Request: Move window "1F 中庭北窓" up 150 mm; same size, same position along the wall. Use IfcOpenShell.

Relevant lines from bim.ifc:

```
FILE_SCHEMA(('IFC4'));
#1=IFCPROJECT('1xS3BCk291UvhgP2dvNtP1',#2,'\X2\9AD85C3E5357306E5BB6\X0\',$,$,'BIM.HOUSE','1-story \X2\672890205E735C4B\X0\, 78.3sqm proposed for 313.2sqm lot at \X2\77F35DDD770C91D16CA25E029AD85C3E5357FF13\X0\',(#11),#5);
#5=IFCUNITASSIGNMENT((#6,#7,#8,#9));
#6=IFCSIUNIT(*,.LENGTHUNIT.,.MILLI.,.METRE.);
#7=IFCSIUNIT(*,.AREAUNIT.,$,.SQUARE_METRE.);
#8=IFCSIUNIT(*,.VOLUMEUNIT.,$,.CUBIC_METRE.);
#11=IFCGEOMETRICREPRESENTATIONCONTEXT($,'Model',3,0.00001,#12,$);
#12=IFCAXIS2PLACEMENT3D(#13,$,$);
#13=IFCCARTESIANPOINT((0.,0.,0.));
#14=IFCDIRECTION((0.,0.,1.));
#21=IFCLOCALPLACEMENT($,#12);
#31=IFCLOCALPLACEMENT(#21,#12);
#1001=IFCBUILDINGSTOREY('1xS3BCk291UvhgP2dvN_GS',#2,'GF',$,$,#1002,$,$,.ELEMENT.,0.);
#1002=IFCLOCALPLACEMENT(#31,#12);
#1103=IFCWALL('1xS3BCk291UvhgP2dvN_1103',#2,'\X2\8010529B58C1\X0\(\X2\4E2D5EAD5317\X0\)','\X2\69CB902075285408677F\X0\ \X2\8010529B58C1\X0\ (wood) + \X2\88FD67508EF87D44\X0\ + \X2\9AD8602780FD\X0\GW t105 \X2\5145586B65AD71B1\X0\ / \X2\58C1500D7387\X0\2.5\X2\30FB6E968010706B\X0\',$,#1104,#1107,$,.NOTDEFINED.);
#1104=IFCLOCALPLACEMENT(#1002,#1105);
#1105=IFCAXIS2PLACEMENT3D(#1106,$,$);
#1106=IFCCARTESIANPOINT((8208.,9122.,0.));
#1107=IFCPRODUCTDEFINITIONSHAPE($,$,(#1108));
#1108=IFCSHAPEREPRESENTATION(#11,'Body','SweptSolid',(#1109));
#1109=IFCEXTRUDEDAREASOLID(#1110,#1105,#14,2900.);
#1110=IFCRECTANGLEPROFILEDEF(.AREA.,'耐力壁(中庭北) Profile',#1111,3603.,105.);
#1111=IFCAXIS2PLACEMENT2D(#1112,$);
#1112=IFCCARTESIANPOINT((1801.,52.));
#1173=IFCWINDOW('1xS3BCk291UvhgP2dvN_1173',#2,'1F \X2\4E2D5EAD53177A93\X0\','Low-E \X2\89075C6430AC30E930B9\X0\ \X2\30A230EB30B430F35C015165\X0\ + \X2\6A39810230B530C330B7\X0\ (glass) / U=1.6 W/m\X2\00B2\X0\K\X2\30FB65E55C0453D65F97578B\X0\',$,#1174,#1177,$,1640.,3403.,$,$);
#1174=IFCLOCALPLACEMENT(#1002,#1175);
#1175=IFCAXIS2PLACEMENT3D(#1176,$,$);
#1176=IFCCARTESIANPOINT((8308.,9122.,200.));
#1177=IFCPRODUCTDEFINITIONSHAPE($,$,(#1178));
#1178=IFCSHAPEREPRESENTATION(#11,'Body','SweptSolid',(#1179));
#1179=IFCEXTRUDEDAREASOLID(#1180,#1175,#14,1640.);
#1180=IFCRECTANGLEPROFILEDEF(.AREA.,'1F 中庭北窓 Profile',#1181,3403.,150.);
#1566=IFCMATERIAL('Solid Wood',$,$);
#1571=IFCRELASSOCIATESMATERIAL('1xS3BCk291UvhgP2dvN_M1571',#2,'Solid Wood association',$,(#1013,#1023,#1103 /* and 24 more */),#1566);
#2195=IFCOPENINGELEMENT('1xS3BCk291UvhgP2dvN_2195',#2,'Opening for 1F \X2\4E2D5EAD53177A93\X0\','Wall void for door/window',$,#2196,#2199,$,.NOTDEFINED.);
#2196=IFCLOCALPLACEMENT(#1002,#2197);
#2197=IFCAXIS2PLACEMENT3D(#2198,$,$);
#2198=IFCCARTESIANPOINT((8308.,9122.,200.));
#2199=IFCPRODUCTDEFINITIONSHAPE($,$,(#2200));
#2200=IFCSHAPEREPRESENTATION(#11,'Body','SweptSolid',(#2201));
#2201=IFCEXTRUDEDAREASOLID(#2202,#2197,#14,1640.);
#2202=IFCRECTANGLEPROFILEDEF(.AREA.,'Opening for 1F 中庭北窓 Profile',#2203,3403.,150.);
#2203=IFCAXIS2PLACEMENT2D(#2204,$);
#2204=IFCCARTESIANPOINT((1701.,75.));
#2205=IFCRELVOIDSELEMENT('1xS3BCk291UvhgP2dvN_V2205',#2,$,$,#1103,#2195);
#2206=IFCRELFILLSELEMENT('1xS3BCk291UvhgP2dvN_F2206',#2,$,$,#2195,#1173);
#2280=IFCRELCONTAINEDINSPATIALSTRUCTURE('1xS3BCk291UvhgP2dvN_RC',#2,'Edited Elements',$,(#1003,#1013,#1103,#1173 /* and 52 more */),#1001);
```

```python
import numpy as np
import ifcopenshell
import ifcopenshell.api.geometry
import ifcopenshell.util.placement
import ifcopenshell.util.unit

model = ifcopenshell.open("bim.ifc")
unit_scale = ifcopenshell.util.unit.calculate_unit_scale(model)

window = model.by_guid("1xS3BCk291UvhgP2dvN_1173")
opening = window.FillsVoids[0].RelatingOpeningElement
dz = 0.15 / unit_scale

shift = np.array([0.0, 0.0, dz])
# The window is not placed relative to its opening, so move both.
for product in (opening, window):
    matrix = ifcopenshell.util.placement.get_local_placement(product.ObjectPlacement)
    matrix[:3, 3] += shift
    ifcopenshell.api.geometry.edit_object_placement(model, product=product, matrix=matrix, is_si=False)

print(f"moved by {dz * unit_scale:+.3f} m")

model.write("bim_updated.ifc")
```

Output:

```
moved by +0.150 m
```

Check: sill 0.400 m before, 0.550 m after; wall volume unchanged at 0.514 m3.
